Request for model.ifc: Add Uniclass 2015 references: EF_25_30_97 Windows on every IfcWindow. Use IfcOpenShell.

First a look at what the model holds.

```python
import ifcopenshell

model = ifcopenshell.open("model.ifc")
print(model.schema)
print("classifications:", [c.Name for c in model.by_type("IfcClassification")])
for ifc_class in ("IfcDoor", "IfcRoof", "IfcStair", "IfcWall", "IfcWindow"):
    print(ifc_class, len(model.by_type(ifc_class)))
```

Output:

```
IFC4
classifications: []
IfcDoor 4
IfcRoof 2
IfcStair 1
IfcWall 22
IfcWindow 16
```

```python
import ifcopenshell
import ifcopenshell.api.classification

model = ifcopenshell.open("model.ifc")

system = ifcopenshell.api.classification.add_classification(model, classification="Uniclass 2015")

codes = {
    "IfcWindow": ("EF_25_30_97", "Windows"),
}
for ifc_class, (code, name) in codes.items():
    products = model.by_type(ifc_class)
    ifcopenshell.api.classification.add_reference(
        model, products=products, classification=system, identification=code, name=name
    )
    print(code, len(products))

model.write("model_edited.ifc")
```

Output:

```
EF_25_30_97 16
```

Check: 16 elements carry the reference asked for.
